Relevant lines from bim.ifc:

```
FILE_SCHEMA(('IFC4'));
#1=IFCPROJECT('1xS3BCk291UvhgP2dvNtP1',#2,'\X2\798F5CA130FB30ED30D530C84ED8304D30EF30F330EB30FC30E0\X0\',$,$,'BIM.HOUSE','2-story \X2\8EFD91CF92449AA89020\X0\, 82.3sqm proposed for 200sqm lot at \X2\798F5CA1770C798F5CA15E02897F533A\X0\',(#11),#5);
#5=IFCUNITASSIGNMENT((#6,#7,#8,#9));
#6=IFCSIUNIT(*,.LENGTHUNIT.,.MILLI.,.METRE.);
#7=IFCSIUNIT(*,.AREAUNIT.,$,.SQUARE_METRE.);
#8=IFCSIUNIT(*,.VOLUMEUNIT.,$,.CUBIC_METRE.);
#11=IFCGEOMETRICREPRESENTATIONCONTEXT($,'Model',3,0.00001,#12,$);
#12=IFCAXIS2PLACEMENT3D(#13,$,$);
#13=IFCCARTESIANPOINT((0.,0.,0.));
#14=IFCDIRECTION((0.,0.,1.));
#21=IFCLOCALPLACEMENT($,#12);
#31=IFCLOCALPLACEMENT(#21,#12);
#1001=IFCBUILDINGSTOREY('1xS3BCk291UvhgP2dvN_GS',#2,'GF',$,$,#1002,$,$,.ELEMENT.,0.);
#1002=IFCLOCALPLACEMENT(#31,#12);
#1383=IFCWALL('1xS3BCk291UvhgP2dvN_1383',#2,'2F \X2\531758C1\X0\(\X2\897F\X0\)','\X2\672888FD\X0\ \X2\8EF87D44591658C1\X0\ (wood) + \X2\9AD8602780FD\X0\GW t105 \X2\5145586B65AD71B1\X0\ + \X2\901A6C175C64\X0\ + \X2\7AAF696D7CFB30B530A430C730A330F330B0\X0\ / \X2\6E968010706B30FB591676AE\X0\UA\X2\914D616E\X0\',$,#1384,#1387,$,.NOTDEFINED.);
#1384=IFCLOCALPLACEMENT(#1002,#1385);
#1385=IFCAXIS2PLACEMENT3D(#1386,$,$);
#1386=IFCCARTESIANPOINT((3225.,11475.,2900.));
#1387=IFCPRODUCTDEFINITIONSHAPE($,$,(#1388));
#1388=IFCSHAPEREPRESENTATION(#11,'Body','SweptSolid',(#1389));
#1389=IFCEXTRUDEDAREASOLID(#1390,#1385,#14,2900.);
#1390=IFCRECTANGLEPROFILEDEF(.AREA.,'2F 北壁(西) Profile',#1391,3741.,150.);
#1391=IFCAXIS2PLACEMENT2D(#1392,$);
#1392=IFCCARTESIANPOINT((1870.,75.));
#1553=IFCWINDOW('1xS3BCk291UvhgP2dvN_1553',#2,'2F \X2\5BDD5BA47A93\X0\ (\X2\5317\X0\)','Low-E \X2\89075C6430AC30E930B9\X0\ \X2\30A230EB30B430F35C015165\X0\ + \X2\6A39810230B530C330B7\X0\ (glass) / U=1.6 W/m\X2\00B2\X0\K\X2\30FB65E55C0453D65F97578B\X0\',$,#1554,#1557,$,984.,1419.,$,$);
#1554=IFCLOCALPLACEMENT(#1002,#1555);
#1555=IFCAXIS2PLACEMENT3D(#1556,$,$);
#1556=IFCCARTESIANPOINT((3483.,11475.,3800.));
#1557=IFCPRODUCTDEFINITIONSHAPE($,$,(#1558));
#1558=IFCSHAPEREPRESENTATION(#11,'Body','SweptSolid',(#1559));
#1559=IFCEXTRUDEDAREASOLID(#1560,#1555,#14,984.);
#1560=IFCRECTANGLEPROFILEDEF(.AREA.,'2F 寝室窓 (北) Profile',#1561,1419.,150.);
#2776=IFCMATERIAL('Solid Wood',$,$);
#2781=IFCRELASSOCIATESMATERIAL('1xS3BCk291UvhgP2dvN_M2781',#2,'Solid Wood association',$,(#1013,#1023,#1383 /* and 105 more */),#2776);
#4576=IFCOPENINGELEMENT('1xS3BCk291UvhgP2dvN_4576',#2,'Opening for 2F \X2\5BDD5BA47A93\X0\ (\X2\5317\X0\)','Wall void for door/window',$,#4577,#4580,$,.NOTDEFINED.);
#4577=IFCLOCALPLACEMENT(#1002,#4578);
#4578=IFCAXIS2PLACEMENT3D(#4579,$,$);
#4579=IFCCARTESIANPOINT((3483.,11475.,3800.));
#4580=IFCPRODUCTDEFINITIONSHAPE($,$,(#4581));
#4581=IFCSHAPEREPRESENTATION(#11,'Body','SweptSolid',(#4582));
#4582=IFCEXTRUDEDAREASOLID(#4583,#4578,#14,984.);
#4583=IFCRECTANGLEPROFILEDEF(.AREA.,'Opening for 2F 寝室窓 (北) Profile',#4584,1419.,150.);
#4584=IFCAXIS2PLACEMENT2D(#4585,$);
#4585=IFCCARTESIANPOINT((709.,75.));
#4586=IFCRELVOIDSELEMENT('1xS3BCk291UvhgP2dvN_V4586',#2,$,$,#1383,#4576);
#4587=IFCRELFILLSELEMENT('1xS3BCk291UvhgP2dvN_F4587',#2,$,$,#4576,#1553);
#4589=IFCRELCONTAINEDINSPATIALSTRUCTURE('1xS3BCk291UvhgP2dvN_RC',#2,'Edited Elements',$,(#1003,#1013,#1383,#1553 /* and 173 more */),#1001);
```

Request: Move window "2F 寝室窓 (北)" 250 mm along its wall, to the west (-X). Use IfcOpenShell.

```python
import ifcopenshell
import ifcopenshell.api.geometry
import ifcopenshell.util.placement
import ifcopenshell.util.unit

model = ifcopenshell.open("bim.ifc")
unit_scale = ifcopenshell.util.unit.calculate_unit_scale(model)

window = model.by_guid("1xS3BCk291UvhgP2dvN_1553")
opening = window.FillsVoids[0].RelatingOpeningElement
wall = opening.VoidsElements[0].RelatingBuildingElement

wall_matrix = ifcopenshell.util.placement.get_local_placement(wall.ObjectPlacement)
shift = wall_matrix[:3, 0] * -0.25 / unit_scale
before = ifcopenshell.util.placement.get_local_placement(window.ObjectPlacement)[:3, 3].copy()

# The window is not placed relative to its opening, so move both.
for product in (opening, window):
    matrix = ifcopenshell.util.placement.get_local_placement(product.ObjectPlacement)
    matrix[:3, 3] += shift
    ifcopenshell.api.geometry.edit_object_placement(model, product=product, matrix=matrix, is_si=False)

after = ifcopenshell.util.placement.get_local_placement(window.ObjectPlacement)[:3, 3]
print("window moved by", (after - before).round(3) + 0.0)

model.write("bim_v2.ifc")
```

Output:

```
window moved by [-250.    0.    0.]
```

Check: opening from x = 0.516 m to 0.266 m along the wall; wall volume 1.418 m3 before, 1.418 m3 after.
